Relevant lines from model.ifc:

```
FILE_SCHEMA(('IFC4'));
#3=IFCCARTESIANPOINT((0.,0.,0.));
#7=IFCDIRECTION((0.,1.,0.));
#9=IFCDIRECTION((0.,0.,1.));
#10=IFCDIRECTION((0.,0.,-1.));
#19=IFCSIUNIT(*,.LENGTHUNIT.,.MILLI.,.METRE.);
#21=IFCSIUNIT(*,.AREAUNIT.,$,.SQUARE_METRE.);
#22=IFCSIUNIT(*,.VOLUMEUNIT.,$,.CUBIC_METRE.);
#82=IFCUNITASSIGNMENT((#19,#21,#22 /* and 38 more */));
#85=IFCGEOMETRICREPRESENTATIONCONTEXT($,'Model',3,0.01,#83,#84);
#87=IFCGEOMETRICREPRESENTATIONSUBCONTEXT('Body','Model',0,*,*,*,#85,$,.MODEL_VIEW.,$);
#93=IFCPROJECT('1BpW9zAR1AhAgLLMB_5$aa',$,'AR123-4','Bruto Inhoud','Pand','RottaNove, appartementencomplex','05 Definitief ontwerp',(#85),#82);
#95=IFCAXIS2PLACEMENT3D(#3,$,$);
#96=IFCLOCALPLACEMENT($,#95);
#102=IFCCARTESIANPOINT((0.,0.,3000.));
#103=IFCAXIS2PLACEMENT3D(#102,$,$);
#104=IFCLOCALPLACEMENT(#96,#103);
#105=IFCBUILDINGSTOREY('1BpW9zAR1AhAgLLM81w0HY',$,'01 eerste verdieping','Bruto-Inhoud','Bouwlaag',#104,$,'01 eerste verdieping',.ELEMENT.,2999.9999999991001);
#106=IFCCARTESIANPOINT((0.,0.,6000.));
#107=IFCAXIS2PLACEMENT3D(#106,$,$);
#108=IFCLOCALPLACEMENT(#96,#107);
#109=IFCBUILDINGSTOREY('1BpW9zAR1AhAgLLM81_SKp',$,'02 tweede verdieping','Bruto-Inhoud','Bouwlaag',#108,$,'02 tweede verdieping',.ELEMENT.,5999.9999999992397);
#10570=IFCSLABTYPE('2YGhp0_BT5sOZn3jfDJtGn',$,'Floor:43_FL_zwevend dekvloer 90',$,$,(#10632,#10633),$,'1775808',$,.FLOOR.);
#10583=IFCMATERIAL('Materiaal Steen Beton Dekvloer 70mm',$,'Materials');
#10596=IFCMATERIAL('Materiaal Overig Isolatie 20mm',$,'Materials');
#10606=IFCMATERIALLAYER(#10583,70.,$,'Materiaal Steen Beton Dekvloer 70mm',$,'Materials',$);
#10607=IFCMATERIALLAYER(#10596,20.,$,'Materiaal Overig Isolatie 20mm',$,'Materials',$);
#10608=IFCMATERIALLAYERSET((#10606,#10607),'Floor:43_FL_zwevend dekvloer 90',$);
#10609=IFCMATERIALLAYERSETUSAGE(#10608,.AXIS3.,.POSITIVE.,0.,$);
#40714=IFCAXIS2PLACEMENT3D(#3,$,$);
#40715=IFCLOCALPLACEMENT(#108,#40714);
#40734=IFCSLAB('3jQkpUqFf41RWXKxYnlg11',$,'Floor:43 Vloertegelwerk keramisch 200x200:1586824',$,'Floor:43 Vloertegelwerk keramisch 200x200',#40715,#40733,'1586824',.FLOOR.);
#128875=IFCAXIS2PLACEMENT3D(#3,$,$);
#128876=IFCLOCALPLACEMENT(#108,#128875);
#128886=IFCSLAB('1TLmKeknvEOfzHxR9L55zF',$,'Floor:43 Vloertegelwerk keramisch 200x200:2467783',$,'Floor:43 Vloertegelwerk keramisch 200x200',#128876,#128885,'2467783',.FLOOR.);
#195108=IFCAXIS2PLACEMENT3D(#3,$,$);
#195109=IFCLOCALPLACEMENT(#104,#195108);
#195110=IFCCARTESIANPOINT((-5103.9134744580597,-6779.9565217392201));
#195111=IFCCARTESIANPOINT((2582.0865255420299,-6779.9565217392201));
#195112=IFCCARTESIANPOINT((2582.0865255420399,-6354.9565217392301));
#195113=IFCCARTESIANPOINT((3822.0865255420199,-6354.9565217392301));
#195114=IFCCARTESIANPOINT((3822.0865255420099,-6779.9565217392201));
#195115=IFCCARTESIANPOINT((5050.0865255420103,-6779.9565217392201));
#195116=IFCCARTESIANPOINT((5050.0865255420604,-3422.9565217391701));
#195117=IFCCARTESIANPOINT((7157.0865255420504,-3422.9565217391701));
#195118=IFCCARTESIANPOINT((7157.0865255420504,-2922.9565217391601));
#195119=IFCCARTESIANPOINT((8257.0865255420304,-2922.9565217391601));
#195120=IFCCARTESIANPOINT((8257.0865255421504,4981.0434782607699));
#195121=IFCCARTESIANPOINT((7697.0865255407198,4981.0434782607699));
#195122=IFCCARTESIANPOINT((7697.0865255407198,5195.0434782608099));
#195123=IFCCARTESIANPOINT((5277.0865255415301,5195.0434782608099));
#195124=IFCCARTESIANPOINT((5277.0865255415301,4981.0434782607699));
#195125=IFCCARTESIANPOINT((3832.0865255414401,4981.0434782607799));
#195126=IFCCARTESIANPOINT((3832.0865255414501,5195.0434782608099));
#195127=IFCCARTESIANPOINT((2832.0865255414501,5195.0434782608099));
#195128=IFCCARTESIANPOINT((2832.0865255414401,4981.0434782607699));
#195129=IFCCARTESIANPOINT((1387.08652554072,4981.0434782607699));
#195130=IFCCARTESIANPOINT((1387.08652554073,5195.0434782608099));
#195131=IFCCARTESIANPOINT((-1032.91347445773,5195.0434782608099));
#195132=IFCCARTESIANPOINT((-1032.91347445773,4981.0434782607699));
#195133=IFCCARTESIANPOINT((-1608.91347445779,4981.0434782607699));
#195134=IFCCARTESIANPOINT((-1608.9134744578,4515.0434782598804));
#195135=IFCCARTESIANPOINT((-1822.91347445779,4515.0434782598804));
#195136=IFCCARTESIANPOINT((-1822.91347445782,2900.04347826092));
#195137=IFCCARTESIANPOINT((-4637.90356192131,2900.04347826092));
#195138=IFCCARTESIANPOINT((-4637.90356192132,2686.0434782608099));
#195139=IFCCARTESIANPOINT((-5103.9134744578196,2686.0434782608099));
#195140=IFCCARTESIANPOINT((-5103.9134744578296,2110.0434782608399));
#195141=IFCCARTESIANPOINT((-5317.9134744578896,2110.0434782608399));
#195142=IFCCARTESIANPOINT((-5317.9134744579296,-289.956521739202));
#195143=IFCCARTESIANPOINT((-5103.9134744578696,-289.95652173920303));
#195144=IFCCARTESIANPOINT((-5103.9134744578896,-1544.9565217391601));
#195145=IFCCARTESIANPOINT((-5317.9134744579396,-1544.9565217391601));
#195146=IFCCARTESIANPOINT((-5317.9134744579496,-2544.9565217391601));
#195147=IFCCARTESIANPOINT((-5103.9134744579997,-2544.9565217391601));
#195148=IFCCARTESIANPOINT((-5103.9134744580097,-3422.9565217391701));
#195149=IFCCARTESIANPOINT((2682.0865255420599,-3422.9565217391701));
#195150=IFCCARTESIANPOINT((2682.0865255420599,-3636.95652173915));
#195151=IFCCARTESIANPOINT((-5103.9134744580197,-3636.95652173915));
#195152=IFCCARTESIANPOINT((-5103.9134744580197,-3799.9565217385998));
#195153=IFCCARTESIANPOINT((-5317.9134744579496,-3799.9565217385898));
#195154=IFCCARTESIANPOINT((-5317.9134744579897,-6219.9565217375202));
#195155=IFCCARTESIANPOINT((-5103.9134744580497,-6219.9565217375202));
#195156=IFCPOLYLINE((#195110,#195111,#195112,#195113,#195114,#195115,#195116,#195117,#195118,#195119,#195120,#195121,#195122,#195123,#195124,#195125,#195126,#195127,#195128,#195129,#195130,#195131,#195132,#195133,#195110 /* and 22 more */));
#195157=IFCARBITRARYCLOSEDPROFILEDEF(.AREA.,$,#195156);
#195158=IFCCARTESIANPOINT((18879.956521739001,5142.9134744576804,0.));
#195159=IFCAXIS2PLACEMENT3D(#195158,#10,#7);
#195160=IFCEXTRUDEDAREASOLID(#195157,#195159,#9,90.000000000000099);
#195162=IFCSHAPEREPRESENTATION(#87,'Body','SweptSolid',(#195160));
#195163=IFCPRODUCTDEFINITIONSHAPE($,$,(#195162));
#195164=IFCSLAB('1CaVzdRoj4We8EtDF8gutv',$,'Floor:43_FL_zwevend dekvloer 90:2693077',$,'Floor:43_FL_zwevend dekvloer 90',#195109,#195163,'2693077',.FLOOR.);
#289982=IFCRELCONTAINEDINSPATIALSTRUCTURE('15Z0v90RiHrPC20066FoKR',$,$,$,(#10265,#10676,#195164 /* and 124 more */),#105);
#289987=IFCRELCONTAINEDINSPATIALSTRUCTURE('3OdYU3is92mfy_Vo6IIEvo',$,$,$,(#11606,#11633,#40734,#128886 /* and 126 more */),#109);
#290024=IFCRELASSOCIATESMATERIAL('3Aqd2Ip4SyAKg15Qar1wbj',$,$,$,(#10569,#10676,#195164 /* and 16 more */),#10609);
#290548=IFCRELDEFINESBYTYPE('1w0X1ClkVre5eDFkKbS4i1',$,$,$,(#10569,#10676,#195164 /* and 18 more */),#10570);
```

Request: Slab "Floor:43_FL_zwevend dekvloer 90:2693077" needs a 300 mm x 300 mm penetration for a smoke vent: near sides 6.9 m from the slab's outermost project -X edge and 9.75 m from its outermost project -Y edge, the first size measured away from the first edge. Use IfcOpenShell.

```python
import numpy as np
import ifcopenshell
import ifcopenshell.api.feature
import ifcopenshell.api.geometry
import ifcopenshell.api.root
import ifcopenshell.geom
import ifcopenshell.util.placement
import ifcopenshell.util.representation
import ifcopenshell.util.shape
import ifcopenshell.util.unit

model = ifcopenshell.open("model.ifc")
unit_scale = ifcopenshell.util.unit.calculate_unit_scale(model)
settings = ifcopenshell.geom.settings()


def volume(element):
    """Net volume in cubic metres, openings subtracted."""
    shape = ifcopenshell.geom.create_shape(settings, element)
    return ifcopenshell.util.shape.get_volume(shape.geometry)


slab = model.by_id(195164)
before = volume(slab)

# Extent in the slab's own axes, in metres. The edges named are its -X and -Y sides.
slab_shape = ifcopenshell.geom.create_shape(settings, slab)
vertices = ifcopenshell.util.shape.get_vertices(slab_shape.geometry)
x_min, y_min, bottom = vertices.min(axis=0)
top = vertices[:, 2].max()

opening = ifcopenshell.api.root.create_entity(model, ifc_class="IfcOpeningElement", name="Smoke vent opening", predefined_type="OPENING")
context = ifcopenshell.util.representation.get_context(model, "Model", "Body", "MODEL_VIEW")
width, depth = 0.3, 0.3
outline = [(0.0, 0.0), (width, 0.0), (width, depth), (0.0, depth), (0.0, 0.0)]
# Overshoot both faces by 50 mm so the cut is clean.
shape = ifcopenshell.api.geometry.add_slab_representation(
    model, context=context, depth=top - bottom + 0.1, polyline=outline
)
ifcopenshell.api.geometry.assign_representation(model, product=opening, representation=shape)

matrix = ifcopenshell.util.placement.get_local_placement(slab.ObjectPlacement)
matrix[:, 3] = matrix @ np.append(np.array([x_min + 6.9, y_min + 9.75, bottom - 0.05]) / unit_scale, 1.0)
ifcopenshell.api.geometry.edit_object_placement(model, product=opening, matrix=matrix, is_si=False)
ifcopenshell.api.feature.add_feature(model, feature=opening, element=slab)

after = volume(slab)

print(f"slab volume {before:.3f} -> {after:.3f} m3")

model.write("model-out.ifc")
```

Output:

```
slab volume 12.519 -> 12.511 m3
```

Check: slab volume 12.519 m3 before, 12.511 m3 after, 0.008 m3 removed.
